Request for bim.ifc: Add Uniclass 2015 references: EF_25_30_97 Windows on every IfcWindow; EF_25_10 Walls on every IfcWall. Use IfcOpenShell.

First a look at what the model holds.

```python
import ifcopenshell

model = ifcopenshell.open("bim.ifc")
print(model.schema)
print("classifications:", [c.Name for c in model.by_type("IfcClassification")])
for ifc_class in ("IfcDoor", "IfcRoof", "IfcStair", "IfcWall", "IfcWindow"):
    print(ifc_class, len(model.by_type(ifc_class)))
```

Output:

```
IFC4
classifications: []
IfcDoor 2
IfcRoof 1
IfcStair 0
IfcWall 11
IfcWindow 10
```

```python
import ifcopenshell
import ifcopenshell.api.classification

model = ifcopenshell.open("bim.ifc")

system = ifcopenshell.api.classification.add_classification(model, classification="Uniclass 2015")

codes = {
    "IfcWindow": ("EF_25_30_97", "Windows"),
    "IfcWall": ("EF_25_10", "Walls"),
}
for ifc_class, (code, name) in codes.items():
    products = model.by_type(ifc_class)
    ifcopenshell.api.classification.add_reference(
        model, products=products, classification=system, identification=code, name=name
    )
    print(code, len(products))

model.write("bim_updated.ifc")
```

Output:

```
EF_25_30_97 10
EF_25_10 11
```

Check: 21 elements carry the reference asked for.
